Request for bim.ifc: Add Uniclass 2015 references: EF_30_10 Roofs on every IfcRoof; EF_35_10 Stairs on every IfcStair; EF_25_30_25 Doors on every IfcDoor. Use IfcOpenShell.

First a look at what the model holds.

```python
import ifcopenshell

model = ifcopenshell.open("bim.ifc")
print(model.schema)
print("classifications:", [c.Name for c in model.by_type("IfcClassification")])
for ifc_class in ("IfcDoor", "IfcRoof", "IfcStair", "IfcWall", "IfcWindow"):
    print(ifc_class, len(model.by_type(ifc_class)))
```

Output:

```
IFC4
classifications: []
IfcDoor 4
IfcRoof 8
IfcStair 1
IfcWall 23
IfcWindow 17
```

```python
import ifcopenshell
import ifcopenshell.api.classification

model = ifcopenshell.open("bim.ifc")

system = ifcopenshell.api.classification.add_classification(model, classification="Uniclass 2015")

codes = {
    "IfcRoof": ("EF_30_10", "Roofs"),
    "IfcStair": ("EF_35_10", "Stairs"),
    "IfcDoor": ("EF_25_30_25", "Doors"),
}
for ifc_class, (code, name) in codes.items():
    products = model.by_type(ifc_class)
    ifcopenshell.api.classification.add_reference(
        model, products=products, classification=system, identification=code, name=name
    )
    print(code, len(products))

model.write("bim_edited.ifc")
```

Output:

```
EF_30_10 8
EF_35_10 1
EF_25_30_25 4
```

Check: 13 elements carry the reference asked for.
